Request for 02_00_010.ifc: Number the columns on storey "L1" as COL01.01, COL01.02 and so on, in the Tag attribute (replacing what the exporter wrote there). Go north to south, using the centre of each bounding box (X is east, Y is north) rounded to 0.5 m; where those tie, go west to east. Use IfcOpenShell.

First a look at what the model holds.

```python
import ifcopenshell
import ifcopenshell.util.element
import ifcopenshell.util.placement

model = ifcopenshell.open("02_00_010.ifc")
print(model.schema)
storey = next(s for s in model.by_type("IfcBuildingStorey") if s.Name == "L1")
columns = [e for e in ifcopenshell.util.element.get_decomposition(storey) if e.is_a("IfcColumn")]
for e in sorted(columns, key=lambda e: e.id()):
    origin = ifcopenshell.util.placement.get_local_placement(e.ObjectPlacement)[:3, 3]
    print(e.id(), e.Tag, e.Name, origin.round(2) + 0.0, sep=" | ")
```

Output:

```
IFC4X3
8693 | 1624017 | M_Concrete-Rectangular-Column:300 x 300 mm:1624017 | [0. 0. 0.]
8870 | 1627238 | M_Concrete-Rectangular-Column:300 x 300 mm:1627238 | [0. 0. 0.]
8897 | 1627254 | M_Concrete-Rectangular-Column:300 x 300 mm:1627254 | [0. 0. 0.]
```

```python
import ifcopenshell
import ifcopenshell.geom
import ifcopenshell.util.element
import ifcopenshell.util.shape

model = ifcopenshell.open("02_00_010.ifc")
settings = ifcopenshell.geom.settings()
settings.set("use-world-coords", True)


def centre(element):
    shape = ifcopenshell.geom.create_shape(settings, element)
    return ifcopenshell.util.shape.get_bbox_centroid(shape.geometry)


storey = next(s for s in model.by_type("IfcBuildingStorey") if s.Name == "L1")
columns = [e for e in ifcopenshell.util.element.get_decomposition(storey) if e.is_a("IfcColumn")]

# Insertion points can sit at a corner or the storey origin, so sort by the geometry (in metres).
centres = {e: centre(e) for e in columns}
columns.sort(key=lambda e: (-round(centres[e][1] / 0.5), centres[e][0]))

for i, e in enumerate(columns, start=1):
    number = f"COL01.{i:02d}"
    e.Tag = number
    print(e.id(), number)

model.write("02_00_010_v2.ifc")
```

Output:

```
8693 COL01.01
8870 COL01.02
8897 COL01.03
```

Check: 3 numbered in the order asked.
